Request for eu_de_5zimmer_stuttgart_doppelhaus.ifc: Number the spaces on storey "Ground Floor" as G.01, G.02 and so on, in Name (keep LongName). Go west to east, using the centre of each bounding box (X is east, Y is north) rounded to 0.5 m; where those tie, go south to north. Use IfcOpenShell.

First a look at what the model holds.

```python
import ifcopenshell
import ifcopenshell.util.element
import ifcopenshell.util.placement

model = ifcopenshell.open("eu_de_5zimmer_stuttgart_doppelhaus.ifc")
print(model.schema)
storey = next(s for s in model.by_type("IfcBuildingStorey") if s.Name == "Ground Floor")
spaces = [e for e in ifcopenshell.util.element.get_decomposition(storey) if e.is_a("IfcSpace")]
for e in sorted(spaces, key=lambda e: e.id()):
    origin = ifcopenshell.util.placement.get_local_placement(e.ObjectPlacement)[:3, 3]
    print(e.id(), e.Name, e.LongName, origin.round(2) + 0.0, sep=" | ")
```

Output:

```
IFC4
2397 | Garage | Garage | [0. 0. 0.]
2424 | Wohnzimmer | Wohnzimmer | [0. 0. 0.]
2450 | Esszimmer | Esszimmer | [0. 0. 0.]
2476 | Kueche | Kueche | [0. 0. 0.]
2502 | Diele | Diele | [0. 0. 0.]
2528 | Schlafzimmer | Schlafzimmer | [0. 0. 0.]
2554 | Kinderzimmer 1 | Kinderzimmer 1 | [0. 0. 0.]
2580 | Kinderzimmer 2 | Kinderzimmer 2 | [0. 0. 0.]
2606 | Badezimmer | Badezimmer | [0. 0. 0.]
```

```python
import ifcopenshell
import ifcopenshell.geom
import ifcopenshell.util.element
import ifcopenshell.util.shape

model = ifcopenshell.open("eu_de_5zimmer_stuttgart_doppelhaus.ifc")
settings = ifcopenshell.geom.settings()
settings.set("use-world-coords", True)


def centre(element):
    shape = ifcopenshell.geom.create_shape(settings, element)
    return ifcopenshell.util.shape.get_bbox_centroid(shape.geometry)


storey = next(s for s in model.by_type("IfcBuildingStorey") if s.Name == "Ground Floor")
spaces = [e for e in ifcopenshell.util.element.get_decomposition(storey) if e.is_a("IfcSpace")]

# Insertion points can sit at a corner or the storey origin, so sort by the geometry (in metres).
centres = {e: centre(e) for e in spaces}
spaces.sort(key=lambda e: (round(centres[e][0] / 0.5), centres[e][1]))

for i, e in enumerate(spaces, start=1):
    number = f"G.{i:02d}"
    e.Name = number
    print(e.id(), number)

model.write("eu_de_5zimmer_stuttgart_doppelhaus_v2.ifc")
```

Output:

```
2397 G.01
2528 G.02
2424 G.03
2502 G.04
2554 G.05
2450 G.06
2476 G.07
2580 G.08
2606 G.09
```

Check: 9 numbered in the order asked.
